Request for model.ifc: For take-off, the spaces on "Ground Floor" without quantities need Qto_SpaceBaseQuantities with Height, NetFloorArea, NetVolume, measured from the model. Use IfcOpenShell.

First a look at what the model holds.

```python
import ifcopenshell
import ifcopenshell.util.element
import ifcopenshell.util.unit

model = ifcopenshell.open("model.ifc")
print(model.schema)
for unit_type in ("LENGTHUNIT", "AREAUNIT", "VOLUMEUNIT"):
    print(unit_type, ifcopenshell.util.unit.calculate_unit_scale(model, unit_type))
storey = next(s for s in model.by_type("IfcBuildingStorey") if s.Name == "Ground Floor")
spaces = [e for e in ifcopenshell.util.element.get_decomposition(storey) if e.is_a("IfcSpace")]
for e in sorted(spaces, key=lambda e: e.id()):
    print(e.id(), e.is_a(), e.Name, list(ifcopenshell.util.element.get_psets(e, qtos_only=True)), sep=" | ")
```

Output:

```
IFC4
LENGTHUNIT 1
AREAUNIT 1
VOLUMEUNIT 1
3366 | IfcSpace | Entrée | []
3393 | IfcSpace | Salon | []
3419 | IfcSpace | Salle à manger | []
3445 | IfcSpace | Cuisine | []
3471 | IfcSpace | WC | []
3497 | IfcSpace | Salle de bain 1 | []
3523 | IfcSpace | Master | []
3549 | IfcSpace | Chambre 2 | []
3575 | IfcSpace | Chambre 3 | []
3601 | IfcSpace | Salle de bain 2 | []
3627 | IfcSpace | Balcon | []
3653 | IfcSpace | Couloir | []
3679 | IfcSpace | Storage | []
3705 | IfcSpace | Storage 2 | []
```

```python
import ifcopenshell
import ifcopenshell.api.pset
import ifcopenshell.geom
import ifcopenshell.util.element
import ifcopenshell.util.shape
import ifcopenshell.util.unit

model = ifcopenshell.open("model.ifc")
unit_scale = ifcopenshell.util.unit.calculate_unit_scale(model)
area_scale = ifcopenshell.util.unit.calculate_unit_scale(model, "AREAUNIT")
volume_scale = ifcopenshell.util.unit.calculate_unit_scale(model, "VOLUMEUNIT")
settings = ifcopenshell.geom.settings()

storey = next(s for s in model.by_type("IfcBuildingStorey") if s.Name == "Ground Floor")
spaces = [e for e in ifcopenshell.util.element.get_decomposition(storey) if e.is_a("IfcSpace")]

for e in sorted(spaces, key=lambda e: e.id()):
    if ifcopenshell.util.element.get_psets(e, qtos_only=True, should_inherit=False):
        continue
    # Geometry comes back in metres, in the element's own axes.
    shape = ifcopenshell.geom.create_shape(settings, e)
    values = {
        "Height": ifcopenshell.util.shape.get_z(shape.geometry) / unit_scale,
        "NetFloorArea": ifcopenshell.util.shape.get_footprint_area(shape.geometry) / area_scale,
        "NetVolume": ifcopenshell.util.shape.get_volume(shape.geometry) / volume_scale,
    }
    qto = ifcopenshell.api.pset.add_qto(model, product=e, name="Qto_SpaceBaseQuantities")
    ifcopenshell.api.pset.edit_qto(model, qto=qto, properties=values)
    print(e.id(), {k: round(v, 3) for k, v in values.items()})

model.write("model_updated.ifc")
```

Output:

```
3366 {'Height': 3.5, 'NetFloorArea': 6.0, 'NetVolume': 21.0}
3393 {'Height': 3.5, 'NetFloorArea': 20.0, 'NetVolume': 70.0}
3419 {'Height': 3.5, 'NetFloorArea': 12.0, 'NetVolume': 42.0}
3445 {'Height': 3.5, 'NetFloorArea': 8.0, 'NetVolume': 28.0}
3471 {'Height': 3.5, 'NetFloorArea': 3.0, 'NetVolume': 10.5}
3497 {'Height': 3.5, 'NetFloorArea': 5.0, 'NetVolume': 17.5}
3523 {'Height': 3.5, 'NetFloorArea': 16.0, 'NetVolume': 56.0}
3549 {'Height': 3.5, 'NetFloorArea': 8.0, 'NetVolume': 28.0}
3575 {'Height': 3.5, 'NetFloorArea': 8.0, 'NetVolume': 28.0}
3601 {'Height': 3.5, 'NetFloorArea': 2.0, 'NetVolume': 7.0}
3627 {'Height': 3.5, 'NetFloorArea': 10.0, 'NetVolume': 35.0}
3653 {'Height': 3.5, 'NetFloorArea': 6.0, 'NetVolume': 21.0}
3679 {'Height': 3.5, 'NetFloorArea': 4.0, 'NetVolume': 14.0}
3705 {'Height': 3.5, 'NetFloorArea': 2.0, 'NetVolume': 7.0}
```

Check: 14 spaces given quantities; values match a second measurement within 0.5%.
